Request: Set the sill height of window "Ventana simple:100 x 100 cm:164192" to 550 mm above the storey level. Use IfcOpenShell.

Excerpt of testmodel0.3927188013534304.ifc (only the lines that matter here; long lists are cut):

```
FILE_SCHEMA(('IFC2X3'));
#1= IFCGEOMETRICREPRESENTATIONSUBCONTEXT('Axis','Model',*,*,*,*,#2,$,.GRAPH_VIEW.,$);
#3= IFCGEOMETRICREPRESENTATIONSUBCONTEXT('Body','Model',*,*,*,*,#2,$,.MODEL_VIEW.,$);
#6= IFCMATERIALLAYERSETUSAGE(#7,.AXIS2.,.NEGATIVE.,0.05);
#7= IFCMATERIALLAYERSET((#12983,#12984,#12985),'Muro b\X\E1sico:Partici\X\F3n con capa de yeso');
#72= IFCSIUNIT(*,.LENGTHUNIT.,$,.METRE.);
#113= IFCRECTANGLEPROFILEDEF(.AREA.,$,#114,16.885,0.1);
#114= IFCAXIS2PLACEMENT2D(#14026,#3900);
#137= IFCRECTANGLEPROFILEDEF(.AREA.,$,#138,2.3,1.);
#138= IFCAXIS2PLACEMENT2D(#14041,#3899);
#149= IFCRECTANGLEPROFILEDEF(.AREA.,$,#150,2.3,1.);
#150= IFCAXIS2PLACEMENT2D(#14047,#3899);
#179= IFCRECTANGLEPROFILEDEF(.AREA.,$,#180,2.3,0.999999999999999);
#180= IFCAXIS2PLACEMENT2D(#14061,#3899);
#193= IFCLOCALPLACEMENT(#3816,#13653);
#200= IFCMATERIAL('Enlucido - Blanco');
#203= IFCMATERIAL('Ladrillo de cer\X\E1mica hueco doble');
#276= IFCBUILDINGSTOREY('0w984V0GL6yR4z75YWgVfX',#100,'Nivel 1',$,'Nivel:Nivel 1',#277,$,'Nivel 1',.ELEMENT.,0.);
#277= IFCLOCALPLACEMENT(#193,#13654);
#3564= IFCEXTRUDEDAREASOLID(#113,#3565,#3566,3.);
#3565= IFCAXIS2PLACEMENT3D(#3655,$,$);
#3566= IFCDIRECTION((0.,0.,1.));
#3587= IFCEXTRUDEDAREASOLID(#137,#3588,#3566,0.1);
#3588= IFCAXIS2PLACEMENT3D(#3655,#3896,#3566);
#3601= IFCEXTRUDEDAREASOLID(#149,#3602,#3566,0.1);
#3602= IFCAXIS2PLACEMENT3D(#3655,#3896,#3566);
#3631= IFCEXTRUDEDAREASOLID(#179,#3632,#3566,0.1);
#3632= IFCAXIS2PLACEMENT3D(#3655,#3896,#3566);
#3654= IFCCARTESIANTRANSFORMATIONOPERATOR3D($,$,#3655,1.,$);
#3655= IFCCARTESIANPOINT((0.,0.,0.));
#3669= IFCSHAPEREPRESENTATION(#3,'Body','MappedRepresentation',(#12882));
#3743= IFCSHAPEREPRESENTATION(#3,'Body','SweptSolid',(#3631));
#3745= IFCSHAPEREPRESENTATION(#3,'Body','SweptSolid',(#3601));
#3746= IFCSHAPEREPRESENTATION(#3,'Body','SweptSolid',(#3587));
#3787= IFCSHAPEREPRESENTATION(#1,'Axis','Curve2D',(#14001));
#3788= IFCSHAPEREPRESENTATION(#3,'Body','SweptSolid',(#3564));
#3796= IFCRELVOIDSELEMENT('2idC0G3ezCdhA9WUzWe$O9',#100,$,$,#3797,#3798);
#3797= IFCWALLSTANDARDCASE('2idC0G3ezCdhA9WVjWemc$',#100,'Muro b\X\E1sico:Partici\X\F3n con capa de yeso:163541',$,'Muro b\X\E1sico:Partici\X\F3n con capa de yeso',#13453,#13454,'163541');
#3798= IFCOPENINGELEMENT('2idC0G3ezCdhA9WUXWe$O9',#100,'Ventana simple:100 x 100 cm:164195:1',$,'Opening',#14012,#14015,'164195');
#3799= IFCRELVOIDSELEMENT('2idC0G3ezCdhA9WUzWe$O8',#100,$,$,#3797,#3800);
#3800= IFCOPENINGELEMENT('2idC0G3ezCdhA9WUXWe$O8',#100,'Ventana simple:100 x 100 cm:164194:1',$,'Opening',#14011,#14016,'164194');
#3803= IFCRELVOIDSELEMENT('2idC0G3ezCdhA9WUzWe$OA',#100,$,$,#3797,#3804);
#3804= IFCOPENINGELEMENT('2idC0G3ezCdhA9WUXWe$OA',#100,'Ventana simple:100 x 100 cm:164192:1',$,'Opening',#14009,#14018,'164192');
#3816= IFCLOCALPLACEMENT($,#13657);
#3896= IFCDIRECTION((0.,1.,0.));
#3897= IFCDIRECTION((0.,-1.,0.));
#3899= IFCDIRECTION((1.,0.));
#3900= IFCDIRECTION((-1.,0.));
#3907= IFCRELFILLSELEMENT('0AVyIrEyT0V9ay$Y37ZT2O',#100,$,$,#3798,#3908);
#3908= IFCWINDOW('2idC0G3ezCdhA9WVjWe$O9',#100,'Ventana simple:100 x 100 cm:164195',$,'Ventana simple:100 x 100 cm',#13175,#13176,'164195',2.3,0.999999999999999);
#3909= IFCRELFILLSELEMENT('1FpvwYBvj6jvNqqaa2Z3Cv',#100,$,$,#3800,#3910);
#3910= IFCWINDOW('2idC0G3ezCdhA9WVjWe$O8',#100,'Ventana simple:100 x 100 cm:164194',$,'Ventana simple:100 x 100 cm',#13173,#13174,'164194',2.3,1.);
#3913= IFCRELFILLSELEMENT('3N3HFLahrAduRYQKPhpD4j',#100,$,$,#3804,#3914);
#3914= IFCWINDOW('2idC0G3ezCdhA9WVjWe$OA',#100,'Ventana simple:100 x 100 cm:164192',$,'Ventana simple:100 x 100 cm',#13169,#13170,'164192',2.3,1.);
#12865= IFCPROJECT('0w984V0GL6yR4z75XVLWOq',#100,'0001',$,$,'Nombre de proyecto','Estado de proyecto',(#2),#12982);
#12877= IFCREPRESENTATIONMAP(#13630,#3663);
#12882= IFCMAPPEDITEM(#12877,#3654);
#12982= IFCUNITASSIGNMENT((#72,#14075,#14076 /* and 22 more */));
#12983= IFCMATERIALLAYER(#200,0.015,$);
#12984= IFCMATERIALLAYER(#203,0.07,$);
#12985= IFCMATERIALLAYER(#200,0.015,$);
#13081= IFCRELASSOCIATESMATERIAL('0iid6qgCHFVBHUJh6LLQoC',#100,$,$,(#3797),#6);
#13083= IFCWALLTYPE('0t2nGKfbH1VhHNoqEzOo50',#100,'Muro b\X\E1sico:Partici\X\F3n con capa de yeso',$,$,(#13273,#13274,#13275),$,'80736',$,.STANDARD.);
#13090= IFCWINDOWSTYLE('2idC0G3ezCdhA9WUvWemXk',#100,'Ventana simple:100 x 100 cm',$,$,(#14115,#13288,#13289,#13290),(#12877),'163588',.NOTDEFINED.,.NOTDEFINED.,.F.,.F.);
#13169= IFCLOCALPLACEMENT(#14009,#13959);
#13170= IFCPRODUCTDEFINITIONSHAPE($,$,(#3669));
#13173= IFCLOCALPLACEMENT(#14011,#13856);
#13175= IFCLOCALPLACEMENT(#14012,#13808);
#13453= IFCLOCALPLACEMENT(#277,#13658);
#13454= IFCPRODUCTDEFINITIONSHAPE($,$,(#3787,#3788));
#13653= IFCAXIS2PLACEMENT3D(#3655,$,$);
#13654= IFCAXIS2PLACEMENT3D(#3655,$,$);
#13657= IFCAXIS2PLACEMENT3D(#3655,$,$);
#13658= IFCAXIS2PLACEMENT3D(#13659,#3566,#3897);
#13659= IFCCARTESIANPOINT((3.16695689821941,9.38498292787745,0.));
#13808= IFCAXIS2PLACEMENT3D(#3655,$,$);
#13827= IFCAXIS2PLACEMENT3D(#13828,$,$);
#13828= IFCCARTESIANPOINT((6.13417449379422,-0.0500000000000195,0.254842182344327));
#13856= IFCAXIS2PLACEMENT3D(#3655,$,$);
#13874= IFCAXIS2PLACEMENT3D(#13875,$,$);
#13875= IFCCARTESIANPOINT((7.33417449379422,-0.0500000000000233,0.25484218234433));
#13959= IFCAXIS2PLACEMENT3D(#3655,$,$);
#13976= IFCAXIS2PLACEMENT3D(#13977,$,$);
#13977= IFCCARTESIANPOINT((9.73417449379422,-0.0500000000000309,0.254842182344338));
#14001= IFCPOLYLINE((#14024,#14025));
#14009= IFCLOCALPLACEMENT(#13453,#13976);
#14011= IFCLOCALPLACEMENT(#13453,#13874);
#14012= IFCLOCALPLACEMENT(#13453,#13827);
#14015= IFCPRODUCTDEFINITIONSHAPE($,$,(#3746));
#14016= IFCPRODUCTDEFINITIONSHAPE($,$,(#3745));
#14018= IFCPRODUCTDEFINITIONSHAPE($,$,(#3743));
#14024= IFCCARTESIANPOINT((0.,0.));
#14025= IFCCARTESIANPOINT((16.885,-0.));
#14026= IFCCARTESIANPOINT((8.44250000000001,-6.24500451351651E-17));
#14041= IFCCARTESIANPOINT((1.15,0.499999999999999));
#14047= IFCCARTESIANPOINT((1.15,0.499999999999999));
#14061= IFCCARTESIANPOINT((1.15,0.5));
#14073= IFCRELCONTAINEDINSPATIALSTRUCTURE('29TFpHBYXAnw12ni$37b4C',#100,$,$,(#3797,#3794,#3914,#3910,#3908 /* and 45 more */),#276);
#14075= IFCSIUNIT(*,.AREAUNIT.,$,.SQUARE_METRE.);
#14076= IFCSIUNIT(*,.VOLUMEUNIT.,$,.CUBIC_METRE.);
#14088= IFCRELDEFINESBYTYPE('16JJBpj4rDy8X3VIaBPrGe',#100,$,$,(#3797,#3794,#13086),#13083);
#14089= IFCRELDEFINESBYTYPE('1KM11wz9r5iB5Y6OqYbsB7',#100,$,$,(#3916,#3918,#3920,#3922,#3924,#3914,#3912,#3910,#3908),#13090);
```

```python
import numpy as np
import ifcopenshell
import ifcopenshell.api.geometry
import ifcopenshell.geom
import ifcopenshell.util.element
import ifcopenshell.util.placement
import ifcopenshell.util.shape
import ifcopenshell.util.unit

model = ifcopenshell.open("testmodel0.3927188013534304.ifc")
unit_scale = ifcopenshell.util.unit.calculate_unit_scale(model)

window = model.by_id(3914)
opening = window.FillsVoids[0].RelatingOpeningElement
storey = ifcopenshell.util.element.get_container(window, ifc_class="IfcBuildingStorey")
level = ifcopenshell.util.placement.get_local_placement(storey.ObjectPlacement)[2, 3]

# The opening's origin need not be at the sill, so measure its lowest point.
shape = ifcopenshell.geom.create_shape(ifcopenshell.geom.settings(), opening)
bottom = ifcopenshell.util.shape.get_shape_bottom_elevation(shape, shape.geometry) / unit_scale
dz = level + 0.55 / unit_scale - bottom

shift = np.array([0.0, 0.0, dz])
# The window is placed relative to its opening, so it follows when the opening moves.
matrix = ifcopenshell.util.placement.get_local_placement(opening.ObjectPlacement)
matrix[:3, 3] += shift
ifcopenshell.api.geometry.edit_object_placement(
    model, product=opening, matrix=matrix, is_si=False, should_transform_children=True
)

print(f"moved by {dz * unit_scale:+.3f} m")

model.write("testmodel0.3927188013534304_v2.ifc")
```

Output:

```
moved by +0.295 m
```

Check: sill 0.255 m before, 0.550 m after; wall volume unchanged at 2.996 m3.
